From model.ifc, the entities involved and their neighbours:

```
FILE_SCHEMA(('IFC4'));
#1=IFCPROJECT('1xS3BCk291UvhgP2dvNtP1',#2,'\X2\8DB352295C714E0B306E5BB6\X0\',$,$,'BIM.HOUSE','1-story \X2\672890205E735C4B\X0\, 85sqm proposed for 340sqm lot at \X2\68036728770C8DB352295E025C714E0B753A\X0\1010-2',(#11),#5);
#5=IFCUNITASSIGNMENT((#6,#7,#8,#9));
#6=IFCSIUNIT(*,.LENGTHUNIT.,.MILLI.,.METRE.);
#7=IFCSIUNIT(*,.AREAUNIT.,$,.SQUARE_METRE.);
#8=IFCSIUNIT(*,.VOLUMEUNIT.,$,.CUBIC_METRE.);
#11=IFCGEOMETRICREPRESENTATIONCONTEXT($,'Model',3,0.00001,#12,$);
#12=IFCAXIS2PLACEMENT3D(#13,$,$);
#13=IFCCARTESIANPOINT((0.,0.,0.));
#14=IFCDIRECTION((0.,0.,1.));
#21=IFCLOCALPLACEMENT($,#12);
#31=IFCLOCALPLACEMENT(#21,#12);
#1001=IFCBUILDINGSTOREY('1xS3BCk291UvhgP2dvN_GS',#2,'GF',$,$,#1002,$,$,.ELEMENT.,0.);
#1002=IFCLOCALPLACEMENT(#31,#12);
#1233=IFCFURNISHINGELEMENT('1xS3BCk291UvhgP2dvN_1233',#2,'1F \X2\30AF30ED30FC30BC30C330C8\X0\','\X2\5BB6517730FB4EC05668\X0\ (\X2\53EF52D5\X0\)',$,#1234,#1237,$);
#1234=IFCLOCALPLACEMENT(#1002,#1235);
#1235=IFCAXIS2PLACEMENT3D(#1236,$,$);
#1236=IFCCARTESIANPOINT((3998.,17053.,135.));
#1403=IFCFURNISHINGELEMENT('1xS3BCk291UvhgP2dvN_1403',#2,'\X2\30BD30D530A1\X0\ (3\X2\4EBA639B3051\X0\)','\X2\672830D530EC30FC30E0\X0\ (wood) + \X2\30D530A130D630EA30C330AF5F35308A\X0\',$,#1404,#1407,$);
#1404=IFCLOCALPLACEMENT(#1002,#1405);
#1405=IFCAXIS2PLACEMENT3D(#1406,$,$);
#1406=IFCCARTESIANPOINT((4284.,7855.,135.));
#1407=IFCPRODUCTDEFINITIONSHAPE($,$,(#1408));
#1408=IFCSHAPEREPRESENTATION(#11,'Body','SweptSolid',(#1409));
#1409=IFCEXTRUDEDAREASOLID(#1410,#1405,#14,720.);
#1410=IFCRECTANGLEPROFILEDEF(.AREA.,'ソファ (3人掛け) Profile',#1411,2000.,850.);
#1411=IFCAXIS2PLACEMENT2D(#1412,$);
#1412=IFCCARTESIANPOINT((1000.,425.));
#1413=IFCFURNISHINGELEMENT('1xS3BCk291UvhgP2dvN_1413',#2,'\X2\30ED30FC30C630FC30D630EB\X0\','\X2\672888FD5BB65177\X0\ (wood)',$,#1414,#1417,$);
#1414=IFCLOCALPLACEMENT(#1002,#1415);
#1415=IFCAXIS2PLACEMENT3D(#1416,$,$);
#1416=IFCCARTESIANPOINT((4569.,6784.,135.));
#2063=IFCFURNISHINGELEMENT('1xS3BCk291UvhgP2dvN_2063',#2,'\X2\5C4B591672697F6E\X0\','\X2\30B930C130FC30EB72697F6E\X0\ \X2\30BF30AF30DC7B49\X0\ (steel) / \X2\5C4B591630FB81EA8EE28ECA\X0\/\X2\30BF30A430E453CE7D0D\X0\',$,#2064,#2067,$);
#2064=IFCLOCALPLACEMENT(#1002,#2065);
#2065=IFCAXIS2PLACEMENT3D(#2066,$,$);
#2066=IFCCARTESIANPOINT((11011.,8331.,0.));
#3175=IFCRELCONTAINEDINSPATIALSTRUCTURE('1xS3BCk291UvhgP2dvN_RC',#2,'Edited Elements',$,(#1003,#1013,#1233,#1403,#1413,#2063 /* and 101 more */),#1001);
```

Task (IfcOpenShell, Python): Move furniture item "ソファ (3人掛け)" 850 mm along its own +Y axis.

```python
import ifcopenshell
import ifcopenshell.api.geometry
import ifcopenshell.util.placement
import ifcopenshell.util.unit

model = ifcopenshell.open("model.ifc")
unit_scale = ifcopenshell.util.unit.calculate_unit_scale(model)

item = model.by_guid("1xS3BCk291UvhgP2dvN_1403")
matrix = ifcopenshell.util.placement.get_local_placement(item.ObjectPlacement)
matrix[:3, 3] += matrix[:3, 1] * 0.85 / unit_scale
ifcopenshell.api.geometry.edit_object_placement(model, product=item, matrix=matrix, is_si=False)

print(ifcopenshell.util.placement.get_local_placement(item.ObjectPlacement).round(3) + 0.0)

model.write("model_rev.ifc")
```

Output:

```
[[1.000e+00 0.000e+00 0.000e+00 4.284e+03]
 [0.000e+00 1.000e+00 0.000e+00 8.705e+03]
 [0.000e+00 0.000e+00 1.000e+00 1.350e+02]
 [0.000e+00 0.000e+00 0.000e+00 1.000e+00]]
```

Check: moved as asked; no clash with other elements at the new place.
